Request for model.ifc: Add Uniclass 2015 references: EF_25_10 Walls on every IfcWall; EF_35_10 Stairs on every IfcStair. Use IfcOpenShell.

First a look at what the model holds.

```python
import ifcopenshell

model = ifcopenshell.open("model.ifc")
print(model.schema)
print("classifications:", [c.Name for c in model.by_type("IfcClassification")])
for ifc_class in ("IfcDoor", "IfcRoof", "IfcStair", "IfcWall", "IfcWindow"):
    print(ifc_class, len(model.by_type(ifc_class)))
```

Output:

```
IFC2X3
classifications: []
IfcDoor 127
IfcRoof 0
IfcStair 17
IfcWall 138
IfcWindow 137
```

```python
import ifcopenshell
import ifcopenshell.api.classification

model = ifcopenshell.open("model.ifc")

# IFC2X3 requires Source and Edition and has no link from the project to the system.
system = model.create_entity("IfcClassification", Source="NBS", Edition="2015", Name="Uniclass 2015")

codes = {
    "IfcWall": ("EF_25_10", "Walls"),
    "IfcStair": ("EF_35_10", "Stairs"),
}
for ifc_class, (code, name) in codes.items():
    products = model.by_type(ifc_class)
    ifcopenshell.api.classification.add_reference(
        model, products=products, classification=system, identification=code, name=name
    )
    print(code, len(products))

model.write("model_v2.ifc")
```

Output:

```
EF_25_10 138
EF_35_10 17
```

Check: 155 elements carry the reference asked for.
